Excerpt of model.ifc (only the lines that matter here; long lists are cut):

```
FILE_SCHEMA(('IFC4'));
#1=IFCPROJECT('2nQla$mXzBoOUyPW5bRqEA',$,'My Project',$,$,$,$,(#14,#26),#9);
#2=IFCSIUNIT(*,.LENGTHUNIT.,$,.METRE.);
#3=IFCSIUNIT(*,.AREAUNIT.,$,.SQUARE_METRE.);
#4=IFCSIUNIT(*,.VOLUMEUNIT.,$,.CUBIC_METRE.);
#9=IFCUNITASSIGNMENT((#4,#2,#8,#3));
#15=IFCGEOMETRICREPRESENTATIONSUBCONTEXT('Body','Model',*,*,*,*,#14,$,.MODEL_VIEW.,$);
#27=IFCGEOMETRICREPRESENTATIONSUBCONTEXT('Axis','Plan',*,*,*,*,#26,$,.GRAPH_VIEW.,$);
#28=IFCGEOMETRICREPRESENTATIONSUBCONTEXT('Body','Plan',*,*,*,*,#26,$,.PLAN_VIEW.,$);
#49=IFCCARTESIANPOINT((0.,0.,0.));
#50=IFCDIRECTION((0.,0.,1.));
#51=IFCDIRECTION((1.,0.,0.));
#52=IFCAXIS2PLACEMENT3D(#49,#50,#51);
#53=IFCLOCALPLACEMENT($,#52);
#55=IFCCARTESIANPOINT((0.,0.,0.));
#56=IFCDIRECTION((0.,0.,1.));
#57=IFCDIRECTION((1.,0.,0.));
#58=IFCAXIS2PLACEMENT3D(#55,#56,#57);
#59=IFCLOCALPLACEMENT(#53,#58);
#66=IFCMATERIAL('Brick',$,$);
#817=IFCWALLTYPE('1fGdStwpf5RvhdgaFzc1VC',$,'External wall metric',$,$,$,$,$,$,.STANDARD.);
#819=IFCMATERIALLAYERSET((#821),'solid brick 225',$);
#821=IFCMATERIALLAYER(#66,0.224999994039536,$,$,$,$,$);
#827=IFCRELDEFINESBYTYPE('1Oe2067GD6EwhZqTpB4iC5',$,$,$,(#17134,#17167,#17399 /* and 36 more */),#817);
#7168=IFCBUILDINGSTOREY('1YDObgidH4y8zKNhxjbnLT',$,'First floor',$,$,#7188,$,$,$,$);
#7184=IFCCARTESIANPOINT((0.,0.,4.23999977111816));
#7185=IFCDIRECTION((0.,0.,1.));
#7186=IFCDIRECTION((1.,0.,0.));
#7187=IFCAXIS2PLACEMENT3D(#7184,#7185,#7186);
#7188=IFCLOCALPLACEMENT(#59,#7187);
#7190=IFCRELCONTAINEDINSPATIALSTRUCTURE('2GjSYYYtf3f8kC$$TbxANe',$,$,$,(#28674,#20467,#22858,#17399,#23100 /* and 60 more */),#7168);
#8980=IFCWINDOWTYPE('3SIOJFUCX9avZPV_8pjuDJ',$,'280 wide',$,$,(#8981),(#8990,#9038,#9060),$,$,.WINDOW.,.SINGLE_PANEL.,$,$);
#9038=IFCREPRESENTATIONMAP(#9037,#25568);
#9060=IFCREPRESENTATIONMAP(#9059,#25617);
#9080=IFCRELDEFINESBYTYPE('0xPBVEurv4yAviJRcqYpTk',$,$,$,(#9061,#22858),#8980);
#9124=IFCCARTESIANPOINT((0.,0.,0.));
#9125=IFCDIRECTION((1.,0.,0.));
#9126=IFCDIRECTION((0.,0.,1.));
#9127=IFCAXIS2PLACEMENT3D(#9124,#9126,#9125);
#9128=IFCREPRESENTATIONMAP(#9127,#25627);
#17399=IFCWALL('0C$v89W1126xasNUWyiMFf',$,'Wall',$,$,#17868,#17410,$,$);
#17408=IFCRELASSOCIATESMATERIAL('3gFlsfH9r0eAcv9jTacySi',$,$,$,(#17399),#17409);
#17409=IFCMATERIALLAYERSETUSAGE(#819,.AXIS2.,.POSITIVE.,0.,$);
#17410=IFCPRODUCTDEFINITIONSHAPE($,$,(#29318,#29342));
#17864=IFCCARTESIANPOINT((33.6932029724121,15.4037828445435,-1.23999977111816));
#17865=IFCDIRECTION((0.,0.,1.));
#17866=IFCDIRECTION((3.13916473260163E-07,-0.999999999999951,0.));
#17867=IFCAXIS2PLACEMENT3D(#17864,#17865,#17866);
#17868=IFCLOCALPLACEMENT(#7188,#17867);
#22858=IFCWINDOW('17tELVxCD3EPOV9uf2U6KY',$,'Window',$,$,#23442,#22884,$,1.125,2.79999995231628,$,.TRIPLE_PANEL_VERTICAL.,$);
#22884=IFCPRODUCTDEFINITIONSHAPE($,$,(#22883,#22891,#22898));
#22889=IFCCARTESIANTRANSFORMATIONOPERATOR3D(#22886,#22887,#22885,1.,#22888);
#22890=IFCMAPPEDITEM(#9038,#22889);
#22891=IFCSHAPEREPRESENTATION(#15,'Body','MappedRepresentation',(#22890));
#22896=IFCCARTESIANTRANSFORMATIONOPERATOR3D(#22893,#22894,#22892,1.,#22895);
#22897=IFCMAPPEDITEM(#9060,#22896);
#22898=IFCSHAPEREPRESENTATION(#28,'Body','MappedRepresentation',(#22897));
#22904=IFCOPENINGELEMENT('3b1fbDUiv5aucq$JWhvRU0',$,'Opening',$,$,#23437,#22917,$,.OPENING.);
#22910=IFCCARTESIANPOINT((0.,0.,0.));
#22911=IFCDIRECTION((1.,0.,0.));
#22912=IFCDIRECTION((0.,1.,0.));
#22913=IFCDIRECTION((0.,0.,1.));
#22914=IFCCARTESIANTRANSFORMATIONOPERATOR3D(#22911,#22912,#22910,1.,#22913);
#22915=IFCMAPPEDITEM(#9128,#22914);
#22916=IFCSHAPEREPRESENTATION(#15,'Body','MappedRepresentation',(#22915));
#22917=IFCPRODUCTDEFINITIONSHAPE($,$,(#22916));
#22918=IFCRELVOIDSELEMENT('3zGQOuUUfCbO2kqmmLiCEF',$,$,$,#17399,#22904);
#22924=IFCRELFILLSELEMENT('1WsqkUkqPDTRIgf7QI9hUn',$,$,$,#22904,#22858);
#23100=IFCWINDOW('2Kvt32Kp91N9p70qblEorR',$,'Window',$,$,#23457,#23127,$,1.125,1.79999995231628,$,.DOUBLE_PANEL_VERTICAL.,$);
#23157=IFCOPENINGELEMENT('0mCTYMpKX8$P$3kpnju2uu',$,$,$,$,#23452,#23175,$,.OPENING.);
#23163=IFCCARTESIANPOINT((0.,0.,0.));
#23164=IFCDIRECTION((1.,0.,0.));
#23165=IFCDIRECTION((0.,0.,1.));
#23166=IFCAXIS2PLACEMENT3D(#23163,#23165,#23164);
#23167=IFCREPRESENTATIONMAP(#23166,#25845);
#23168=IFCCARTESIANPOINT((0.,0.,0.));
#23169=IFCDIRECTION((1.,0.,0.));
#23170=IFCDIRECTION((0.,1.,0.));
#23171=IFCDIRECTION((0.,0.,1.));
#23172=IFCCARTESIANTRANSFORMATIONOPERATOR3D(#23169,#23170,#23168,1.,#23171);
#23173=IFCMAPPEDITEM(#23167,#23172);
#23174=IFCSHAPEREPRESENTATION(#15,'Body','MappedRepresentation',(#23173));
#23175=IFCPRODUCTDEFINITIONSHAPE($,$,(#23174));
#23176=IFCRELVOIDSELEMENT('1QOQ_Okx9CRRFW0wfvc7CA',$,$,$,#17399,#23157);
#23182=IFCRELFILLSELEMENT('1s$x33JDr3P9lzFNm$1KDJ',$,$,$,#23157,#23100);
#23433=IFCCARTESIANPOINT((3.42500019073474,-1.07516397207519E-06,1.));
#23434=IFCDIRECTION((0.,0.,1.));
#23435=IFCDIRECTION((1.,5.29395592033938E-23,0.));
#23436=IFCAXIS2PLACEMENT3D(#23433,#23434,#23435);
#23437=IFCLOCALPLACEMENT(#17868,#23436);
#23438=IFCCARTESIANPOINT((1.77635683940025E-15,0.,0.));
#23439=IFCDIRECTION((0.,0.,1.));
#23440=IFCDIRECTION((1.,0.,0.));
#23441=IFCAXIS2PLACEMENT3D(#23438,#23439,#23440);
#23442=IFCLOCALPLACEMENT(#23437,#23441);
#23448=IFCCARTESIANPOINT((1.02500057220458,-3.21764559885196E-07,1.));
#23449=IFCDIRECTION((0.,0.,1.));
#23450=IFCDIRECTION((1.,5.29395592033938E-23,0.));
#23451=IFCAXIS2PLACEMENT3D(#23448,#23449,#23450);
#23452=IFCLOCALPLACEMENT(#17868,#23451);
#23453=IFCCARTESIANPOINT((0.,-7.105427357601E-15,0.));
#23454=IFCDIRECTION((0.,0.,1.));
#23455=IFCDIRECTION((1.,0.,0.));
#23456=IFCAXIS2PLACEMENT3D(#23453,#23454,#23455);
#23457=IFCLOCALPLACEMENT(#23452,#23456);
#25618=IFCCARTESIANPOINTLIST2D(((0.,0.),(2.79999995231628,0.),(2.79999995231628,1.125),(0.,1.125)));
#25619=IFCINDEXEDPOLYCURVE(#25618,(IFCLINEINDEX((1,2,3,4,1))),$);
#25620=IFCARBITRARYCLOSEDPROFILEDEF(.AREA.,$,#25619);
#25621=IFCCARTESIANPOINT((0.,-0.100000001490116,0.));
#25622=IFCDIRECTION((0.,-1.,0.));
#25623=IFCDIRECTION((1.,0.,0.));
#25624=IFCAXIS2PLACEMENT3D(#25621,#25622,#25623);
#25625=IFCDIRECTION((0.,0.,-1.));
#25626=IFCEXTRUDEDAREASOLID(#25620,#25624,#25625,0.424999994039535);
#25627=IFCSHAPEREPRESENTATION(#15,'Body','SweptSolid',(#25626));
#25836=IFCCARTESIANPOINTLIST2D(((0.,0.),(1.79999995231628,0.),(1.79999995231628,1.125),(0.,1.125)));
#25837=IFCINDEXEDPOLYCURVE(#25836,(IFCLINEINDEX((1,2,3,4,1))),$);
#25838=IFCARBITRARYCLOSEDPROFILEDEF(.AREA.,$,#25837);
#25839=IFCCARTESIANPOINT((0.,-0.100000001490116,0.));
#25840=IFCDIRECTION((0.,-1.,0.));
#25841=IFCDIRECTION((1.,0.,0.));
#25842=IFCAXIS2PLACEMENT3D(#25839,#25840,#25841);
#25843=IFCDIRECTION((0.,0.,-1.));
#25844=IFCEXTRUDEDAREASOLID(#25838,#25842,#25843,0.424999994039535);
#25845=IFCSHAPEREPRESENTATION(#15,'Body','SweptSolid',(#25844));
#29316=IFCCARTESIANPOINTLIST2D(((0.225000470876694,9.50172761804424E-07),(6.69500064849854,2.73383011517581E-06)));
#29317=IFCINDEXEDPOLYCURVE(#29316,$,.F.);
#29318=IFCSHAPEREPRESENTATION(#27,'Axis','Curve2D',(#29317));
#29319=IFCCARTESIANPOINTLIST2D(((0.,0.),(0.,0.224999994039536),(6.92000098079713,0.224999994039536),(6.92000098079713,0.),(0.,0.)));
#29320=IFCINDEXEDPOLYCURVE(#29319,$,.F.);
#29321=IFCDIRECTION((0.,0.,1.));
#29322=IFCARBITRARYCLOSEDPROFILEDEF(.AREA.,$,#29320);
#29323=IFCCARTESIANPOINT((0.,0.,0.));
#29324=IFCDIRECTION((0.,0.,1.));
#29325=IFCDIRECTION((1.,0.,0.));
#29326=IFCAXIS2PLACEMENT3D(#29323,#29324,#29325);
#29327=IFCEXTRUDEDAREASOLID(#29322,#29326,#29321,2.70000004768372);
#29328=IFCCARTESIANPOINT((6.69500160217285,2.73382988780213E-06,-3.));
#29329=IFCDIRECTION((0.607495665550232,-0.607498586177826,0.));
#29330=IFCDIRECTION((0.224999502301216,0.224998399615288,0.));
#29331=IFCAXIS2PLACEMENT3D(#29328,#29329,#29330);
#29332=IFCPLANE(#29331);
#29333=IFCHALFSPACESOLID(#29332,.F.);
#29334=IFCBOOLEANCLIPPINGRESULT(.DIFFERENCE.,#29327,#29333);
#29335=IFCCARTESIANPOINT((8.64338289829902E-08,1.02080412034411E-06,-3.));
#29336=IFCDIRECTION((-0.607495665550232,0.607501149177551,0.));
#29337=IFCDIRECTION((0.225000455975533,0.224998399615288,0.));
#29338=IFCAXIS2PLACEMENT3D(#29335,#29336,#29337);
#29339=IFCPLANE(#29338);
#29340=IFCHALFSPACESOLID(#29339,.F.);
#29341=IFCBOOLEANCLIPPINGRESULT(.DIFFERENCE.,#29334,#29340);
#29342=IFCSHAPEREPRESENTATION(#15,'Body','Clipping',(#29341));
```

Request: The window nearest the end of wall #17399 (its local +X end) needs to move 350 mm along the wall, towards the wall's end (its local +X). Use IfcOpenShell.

```python
import ifcopenshell
import ifcopenshell.api.geometry
import ifcopenshell.util.placement
import ifcopenshell.util.unit

model = ifcopenshell.open("model.ifc")
unit_scale = ifcopenshell.util.unit.calculate_unit_scale(model)

window = model.by_id(22858)
opening = window.FillsVoids[0].RelatingOpeningElement
wall = opening.VoidsElements[0].RelatingBuildingElement

wall_matrix = ifcopenshell.util.placement.get_local_placement(wall.ObjectPlacement)
shift = wall_matrix[:3, 0] * 0.35 / unit_scale
before = ifcopenshell.util.placement.get_local_placement(window.ObjectPlacement)[:3, 3].copy()

# The window is placed relative to its opening, so it follows when the opening moves.
matrix = ifcopenshell.util.placement.get_local_placement(opening.ObjectPlacement)
matrix[:3, 3] += shift
ifcopenshell.api.geometry.edit_object_placement(
    model, product=opening, matrix=matrix, is_si=False, should_transform_children=True
)

after = ifcopenshell.util.placement.get_local_placement(window.ObjectPlacement)[:3, 3]
print("window moved by", (after - before).round(3) + 0.0)

model.write("model-out.ifc")
```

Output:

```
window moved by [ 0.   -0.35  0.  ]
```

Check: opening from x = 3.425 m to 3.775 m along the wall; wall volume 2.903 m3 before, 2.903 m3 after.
